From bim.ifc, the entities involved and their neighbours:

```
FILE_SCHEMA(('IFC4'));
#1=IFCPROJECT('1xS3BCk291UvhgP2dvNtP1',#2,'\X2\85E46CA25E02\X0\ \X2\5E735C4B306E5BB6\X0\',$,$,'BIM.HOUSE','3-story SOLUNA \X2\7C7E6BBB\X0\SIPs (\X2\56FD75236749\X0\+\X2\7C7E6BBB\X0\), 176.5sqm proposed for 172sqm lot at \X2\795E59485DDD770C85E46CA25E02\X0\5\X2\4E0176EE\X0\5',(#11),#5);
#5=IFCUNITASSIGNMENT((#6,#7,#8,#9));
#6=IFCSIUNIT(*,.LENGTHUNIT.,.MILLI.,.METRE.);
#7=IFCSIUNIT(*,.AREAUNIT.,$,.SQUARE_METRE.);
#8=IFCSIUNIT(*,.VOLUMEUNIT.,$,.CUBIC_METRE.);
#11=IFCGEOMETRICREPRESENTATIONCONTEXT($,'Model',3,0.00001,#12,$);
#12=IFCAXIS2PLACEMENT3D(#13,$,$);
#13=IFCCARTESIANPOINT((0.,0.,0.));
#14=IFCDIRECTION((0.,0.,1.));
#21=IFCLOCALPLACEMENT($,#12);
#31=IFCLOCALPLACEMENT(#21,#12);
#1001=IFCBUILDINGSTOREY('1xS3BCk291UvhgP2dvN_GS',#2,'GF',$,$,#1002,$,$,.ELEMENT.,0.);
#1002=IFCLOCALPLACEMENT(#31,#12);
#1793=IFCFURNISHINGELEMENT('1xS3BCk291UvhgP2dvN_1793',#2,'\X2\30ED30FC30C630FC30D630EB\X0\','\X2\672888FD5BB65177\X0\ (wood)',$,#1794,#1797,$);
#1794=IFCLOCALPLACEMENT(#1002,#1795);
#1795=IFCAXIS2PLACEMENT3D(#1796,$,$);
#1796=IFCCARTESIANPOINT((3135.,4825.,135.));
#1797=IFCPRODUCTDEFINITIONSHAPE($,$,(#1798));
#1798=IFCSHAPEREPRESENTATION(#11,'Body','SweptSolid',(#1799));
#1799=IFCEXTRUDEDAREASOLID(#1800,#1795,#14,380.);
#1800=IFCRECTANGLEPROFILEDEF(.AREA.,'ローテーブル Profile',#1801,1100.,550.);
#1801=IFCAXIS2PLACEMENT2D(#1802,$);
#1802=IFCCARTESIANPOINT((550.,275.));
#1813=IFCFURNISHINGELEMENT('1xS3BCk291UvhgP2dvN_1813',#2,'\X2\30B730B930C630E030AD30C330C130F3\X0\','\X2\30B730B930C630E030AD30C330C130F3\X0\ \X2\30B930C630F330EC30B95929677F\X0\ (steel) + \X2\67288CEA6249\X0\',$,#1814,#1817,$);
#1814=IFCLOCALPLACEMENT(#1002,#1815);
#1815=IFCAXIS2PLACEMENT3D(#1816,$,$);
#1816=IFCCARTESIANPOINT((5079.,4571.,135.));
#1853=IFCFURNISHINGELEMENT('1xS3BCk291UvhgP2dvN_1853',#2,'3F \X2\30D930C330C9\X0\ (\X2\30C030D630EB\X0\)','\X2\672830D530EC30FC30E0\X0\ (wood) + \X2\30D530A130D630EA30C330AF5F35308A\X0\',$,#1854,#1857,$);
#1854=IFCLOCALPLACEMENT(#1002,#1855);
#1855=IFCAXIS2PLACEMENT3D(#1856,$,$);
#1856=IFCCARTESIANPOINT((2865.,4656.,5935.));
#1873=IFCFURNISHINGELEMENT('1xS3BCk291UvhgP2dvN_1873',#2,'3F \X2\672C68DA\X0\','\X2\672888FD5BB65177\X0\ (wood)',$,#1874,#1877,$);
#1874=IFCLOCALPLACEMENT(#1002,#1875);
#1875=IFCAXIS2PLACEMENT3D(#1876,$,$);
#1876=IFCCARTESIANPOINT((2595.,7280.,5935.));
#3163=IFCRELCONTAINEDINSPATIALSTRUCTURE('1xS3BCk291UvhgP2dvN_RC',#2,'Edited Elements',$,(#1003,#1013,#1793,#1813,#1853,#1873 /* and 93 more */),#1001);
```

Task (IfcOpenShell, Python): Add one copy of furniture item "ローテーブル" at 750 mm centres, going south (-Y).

```python
import numpy as np
import ifcopenshell
import ifcopenshell.api.geometry
import ifcopenshell.api.root
import ifcopenshell.util.element
import ifcopenshell.util.placement
import ifcopenshell.util.unit

model = ifcopenshell.open("bim.ifc")
unit_scale = ifcopenshell.util.unit.calculate_unit_scale(model)


def reuse_history(source, copy):
    """copy_class also copies each property set's owner history, people and application; keep the originals."""
    for rel in copy.IsDefinedBy:
        if rel.is_a("IfcRelDefinesByProperties") and (history := rel.RelatingPropertyDefinition.OwnerHistory):
            rel.RelatingPropertyDefinition.OwnerHistory = source.OwnerHistory
            ifcopenshell.util.element.remove_deep2(model, history)


source = model.by_guid("1xS3BCk291UvhgP2dvN_1793")
base = ifcopenshell.util.placement.get_local_placement(source.ObjectPlacement)
step = np.array([0.0, -1.0, 0.0]) * 0.75 / unit_scale

for i in range(1, 2):
    copy = ifcopenshell.api.root.copy_class(model, product=source)
    copy.Representation = ifcopenshell.util.element.copy_deep(
        model, source.Representation, exclude=["IfcGeometricRepresentationContext", "IfcRepresentationMap"]
    )
    reuse_history(source, copy)
    matrix = base.copy()
    matrix[:3, 3] += i * step
    print("added at", matrix[:3, 3].round(3) + 0.0)
    ifcopenshell.api.geometry.edit_object_placement(model, product=copy, matrix=matrix, is_si=False)

model.write("bim_edited.ifc")
```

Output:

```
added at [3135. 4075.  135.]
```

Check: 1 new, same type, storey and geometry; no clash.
